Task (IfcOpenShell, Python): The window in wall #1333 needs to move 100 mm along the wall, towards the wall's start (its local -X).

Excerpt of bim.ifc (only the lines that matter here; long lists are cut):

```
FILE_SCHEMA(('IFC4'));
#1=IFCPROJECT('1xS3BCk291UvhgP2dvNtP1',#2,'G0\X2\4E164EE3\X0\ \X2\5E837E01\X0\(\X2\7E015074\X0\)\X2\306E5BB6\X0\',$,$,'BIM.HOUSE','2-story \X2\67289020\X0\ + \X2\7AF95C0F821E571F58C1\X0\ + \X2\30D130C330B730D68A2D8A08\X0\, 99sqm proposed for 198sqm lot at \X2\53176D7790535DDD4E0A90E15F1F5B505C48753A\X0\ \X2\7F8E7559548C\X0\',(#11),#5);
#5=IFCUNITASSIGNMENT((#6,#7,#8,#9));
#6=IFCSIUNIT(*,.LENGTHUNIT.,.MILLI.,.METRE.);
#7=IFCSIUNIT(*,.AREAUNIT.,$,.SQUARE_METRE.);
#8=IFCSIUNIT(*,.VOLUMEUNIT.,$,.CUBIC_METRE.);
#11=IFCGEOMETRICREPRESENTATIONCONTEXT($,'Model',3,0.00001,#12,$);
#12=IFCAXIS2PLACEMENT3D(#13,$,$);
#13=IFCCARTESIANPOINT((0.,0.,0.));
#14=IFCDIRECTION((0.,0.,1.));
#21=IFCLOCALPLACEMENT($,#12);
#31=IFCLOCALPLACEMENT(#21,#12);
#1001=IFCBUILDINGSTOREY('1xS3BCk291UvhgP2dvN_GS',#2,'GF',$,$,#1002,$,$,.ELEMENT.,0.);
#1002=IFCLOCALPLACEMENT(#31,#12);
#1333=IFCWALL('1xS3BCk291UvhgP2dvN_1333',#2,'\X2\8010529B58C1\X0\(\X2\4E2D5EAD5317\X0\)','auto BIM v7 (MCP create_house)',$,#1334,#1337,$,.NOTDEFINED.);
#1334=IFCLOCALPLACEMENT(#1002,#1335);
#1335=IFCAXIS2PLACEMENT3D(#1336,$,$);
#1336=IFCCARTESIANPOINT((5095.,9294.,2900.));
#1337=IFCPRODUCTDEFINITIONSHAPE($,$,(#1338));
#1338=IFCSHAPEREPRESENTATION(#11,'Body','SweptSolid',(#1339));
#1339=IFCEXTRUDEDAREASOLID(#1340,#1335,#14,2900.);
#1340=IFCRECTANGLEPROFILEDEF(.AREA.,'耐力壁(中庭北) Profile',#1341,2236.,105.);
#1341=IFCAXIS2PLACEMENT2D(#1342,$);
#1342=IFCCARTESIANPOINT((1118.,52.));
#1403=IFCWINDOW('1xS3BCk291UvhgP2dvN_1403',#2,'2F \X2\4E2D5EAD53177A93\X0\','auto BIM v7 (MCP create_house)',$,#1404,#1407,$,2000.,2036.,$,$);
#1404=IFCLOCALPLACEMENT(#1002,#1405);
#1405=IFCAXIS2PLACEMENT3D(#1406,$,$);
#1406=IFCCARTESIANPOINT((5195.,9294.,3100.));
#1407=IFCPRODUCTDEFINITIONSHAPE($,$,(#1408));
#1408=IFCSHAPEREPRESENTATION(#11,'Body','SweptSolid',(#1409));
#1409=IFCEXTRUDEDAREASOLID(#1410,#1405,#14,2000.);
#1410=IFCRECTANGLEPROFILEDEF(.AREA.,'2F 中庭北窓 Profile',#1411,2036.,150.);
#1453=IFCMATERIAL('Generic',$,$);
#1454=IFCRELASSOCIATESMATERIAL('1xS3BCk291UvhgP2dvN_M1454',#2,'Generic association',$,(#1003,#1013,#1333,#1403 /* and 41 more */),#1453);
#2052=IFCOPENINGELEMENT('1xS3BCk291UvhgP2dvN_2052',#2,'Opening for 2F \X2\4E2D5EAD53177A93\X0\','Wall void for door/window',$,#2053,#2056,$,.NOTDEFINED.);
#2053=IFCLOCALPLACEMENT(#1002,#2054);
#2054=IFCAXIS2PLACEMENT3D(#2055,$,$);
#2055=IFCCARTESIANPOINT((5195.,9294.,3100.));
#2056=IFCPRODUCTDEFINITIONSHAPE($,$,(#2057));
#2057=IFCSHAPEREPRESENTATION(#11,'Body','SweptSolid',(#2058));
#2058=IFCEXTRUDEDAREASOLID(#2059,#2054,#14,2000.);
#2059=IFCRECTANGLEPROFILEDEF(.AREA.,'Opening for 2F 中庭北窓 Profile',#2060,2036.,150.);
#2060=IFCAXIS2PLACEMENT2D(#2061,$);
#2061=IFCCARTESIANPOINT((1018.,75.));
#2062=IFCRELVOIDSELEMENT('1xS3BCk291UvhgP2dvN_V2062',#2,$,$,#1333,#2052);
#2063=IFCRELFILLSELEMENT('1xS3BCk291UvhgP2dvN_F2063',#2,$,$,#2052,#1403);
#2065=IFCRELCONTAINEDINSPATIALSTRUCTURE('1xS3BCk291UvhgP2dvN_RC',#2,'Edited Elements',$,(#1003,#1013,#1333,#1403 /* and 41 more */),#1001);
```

```python
import ifcopenshell
import ifcopenshell.api.geometry
import ifcopenshell.util.placement
import ifcopenshell.util.unit

model = ifcopenshell.open("bim.ifc")
unit_scale = ifcopenshell.util.unit.calculate_unit_scale(model)

window = model.by_guid("1xS3BCk291UvhgP2dvN_1403")
opening = window.FillsVoids[0].RelatingOpeningElement
wall = opening.VoidsElements[0].RelatingBuildingElement

wall_matrix = ifcopenshell.util.placement.get_local_placement(wall.ObjectPlacement)
shift = wall_matrix[:3, 0] * -0.1 / unit_scale
before = ifcopenshell.util.placement.get_local_placement(window.ObjectPlacement)[:3, 3].copy()

# The window is not placed relative to its opening, so move both.
for product in (opening, window):
    matrix = ifcopenshell.util.placement.get_local_placement(product.ObjectPlacement)
    matrix[:3, 3] += shift
    ifcopenshell.api.geometry.edit_object_placement(model, product=product, matrix=matrix, is_si=False)

after = ifcopenshell.util.placement.get_local_placement(window.ObjectPlacement)[:3, 3]
print("window moved by", (after - before).round(3) + 0.0)

model.write("bim_v2.ifc")
```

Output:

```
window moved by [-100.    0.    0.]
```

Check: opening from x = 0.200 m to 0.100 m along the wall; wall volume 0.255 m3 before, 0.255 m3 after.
